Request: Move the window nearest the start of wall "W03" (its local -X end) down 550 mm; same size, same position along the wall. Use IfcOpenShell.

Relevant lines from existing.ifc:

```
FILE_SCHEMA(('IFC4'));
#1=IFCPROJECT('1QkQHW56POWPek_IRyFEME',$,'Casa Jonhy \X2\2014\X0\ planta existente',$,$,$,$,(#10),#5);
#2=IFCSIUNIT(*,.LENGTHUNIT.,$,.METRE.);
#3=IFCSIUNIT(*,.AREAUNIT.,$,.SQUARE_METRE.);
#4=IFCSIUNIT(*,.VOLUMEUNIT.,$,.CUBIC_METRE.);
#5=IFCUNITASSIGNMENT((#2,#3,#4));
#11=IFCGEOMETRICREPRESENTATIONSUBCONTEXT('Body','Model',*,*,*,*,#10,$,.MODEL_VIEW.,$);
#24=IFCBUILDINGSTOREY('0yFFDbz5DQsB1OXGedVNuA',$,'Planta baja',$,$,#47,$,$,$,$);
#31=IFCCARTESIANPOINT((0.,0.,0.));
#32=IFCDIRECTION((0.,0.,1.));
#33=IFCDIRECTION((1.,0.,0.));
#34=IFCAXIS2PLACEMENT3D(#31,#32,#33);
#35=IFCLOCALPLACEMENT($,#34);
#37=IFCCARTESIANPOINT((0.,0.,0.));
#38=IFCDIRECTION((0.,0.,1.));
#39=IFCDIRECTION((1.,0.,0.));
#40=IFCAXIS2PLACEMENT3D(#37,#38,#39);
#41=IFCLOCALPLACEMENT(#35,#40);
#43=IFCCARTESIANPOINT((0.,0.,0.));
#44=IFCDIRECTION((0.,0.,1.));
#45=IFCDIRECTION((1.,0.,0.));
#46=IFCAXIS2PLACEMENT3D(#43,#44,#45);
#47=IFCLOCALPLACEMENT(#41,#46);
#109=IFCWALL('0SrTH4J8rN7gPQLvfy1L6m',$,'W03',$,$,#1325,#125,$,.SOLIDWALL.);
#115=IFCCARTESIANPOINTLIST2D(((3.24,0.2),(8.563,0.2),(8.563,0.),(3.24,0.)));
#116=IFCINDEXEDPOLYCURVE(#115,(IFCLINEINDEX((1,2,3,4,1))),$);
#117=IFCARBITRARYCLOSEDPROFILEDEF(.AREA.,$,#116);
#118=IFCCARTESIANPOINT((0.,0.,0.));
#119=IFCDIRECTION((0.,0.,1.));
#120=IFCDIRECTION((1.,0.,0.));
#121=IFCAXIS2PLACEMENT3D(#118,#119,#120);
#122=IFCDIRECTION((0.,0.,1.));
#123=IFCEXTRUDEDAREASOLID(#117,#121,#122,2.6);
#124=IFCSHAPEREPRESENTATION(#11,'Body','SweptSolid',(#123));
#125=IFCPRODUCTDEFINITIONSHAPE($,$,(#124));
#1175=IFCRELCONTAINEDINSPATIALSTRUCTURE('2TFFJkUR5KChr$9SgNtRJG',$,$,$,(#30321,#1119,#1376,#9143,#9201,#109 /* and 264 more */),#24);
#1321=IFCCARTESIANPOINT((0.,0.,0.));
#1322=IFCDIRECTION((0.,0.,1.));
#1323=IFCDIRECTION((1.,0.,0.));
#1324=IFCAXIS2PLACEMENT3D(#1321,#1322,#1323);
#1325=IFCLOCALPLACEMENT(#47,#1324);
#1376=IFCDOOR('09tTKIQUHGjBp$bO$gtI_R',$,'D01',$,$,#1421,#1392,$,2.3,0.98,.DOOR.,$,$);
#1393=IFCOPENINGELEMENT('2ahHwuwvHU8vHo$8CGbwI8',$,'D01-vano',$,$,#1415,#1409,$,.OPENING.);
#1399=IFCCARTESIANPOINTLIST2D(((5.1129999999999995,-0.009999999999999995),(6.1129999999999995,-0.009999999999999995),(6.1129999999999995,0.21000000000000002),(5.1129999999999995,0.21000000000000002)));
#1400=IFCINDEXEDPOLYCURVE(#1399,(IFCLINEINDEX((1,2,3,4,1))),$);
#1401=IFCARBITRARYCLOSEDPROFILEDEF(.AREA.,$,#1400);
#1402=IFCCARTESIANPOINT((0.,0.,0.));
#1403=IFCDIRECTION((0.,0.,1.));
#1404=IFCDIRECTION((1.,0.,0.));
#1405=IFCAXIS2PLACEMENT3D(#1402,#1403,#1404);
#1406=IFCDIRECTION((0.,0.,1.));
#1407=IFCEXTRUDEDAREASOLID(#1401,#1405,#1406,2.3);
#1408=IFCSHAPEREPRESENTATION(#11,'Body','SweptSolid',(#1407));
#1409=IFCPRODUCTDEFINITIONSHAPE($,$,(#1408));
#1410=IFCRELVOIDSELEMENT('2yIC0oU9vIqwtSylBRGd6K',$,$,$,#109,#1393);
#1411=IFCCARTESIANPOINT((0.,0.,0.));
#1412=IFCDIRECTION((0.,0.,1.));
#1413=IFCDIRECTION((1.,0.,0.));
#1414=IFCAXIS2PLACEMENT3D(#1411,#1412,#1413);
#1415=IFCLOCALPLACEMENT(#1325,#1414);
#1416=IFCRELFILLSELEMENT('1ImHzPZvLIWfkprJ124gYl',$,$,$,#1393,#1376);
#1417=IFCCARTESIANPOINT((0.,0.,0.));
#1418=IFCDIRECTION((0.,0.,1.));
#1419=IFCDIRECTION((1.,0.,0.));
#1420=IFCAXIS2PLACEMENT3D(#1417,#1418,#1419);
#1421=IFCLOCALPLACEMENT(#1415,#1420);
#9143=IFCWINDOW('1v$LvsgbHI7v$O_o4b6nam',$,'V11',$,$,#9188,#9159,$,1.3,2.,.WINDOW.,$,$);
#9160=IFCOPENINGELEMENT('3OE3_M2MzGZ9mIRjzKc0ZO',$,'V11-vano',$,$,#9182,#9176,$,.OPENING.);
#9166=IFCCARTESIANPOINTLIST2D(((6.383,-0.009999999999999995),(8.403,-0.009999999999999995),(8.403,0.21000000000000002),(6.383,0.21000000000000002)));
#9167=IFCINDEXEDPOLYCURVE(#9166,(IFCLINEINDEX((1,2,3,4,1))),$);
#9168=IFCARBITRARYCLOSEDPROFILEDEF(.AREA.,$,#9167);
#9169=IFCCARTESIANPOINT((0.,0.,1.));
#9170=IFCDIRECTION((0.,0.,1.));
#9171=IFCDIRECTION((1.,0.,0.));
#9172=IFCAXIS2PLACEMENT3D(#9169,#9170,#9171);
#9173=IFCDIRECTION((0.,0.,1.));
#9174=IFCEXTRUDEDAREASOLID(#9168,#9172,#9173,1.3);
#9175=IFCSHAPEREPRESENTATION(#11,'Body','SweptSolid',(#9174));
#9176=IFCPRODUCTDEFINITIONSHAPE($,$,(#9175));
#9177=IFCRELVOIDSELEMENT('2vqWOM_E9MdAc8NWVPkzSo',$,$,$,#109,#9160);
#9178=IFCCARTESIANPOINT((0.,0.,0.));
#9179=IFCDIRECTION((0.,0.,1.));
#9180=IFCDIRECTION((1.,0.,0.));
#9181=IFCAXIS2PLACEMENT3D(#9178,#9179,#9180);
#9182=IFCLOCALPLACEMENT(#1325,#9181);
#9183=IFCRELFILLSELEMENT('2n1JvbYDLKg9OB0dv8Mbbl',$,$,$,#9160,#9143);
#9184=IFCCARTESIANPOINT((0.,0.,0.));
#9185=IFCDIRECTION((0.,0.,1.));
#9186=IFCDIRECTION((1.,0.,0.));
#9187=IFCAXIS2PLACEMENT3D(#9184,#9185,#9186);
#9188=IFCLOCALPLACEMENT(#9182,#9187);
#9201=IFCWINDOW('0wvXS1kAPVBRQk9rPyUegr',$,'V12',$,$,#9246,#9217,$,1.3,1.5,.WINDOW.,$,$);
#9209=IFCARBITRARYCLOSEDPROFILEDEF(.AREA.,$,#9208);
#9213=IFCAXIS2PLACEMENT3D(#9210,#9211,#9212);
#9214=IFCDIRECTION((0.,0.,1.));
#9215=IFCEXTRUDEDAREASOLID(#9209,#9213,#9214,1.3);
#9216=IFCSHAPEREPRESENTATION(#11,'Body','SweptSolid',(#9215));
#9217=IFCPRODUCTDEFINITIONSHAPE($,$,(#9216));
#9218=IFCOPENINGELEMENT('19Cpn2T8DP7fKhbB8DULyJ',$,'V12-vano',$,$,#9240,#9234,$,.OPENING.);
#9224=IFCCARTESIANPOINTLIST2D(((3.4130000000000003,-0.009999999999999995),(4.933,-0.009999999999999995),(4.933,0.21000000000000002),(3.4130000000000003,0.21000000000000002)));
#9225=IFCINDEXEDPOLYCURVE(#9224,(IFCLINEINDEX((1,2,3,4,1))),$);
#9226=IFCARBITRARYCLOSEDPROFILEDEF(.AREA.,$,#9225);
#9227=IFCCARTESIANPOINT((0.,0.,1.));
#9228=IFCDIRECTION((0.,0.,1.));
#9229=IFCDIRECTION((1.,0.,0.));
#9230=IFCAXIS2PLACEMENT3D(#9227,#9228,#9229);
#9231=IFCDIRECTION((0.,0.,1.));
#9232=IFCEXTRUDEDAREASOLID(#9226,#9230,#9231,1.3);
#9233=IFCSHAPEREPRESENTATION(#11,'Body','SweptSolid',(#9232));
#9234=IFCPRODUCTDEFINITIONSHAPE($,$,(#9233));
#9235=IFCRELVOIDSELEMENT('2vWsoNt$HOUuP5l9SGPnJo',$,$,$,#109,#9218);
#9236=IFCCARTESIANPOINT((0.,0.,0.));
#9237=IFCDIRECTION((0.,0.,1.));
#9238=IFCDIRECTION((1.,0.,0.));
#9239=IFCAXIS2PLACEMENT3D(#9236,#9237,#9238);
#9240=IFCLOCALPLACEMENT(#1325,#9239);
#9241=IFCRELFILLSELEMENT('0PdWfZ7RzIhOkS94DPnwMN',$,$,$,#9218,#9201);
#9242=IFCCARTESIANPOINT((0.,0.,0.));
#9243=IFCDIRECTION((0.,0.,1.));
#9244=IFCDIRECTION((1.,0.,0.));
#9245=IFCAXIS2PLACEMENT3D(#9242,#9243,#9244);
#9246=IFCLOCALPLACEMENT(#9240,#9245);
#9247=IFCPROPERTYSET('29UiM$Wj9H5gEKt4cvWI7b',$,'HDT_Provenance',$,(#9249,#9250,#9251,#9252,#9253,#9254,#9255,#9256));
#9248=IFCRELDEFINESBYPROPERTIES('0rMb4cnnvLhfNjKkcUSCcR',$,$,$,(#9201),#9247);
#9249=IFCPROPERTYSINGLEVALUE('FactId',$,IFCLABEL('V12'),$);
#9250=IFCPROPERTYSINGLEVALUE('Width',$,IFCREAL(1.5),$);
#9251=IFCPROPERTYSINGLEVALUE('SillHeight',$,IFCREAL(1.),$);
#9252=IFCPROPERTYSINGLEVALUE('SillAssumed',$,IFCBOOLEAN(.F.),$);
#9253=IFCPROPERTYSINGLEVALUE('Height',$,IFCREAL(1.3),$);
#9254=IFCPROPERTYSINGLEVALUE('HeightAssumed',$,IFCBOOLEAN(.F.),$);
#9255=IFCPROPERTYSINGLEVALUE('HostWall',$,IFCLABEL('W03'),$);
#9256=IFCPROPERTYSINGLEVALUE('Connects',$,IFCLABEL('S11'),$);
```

```python
import numpy as np
import ifcopenshell
import ifcopenshell.api.geometry
import ifcopenshell.api.pset
import ifcopenshell.util.element
import ifcopenshell.util.placement
import ifcopenshell.util.unit

model = ifcopenshell.open("existing.ifc")
unit_scale = ifcopenshell.util.unit.calculate_unit_scale(model)

window = model.by_guid("0wvXS1kAPVBRQk9rPyUegr")
opening = window.FillsVoids[0].RelatingOpeningElement
dz = -0.55 / unit_scale

shift = np.array([0.0, 0.0, dz])
# The window is placed relative to its opening, so it follows when the opening moves.
matrix = ifcopenshell.util.placement.get_local_placement(opening.ObjectPlacement)
matrix[:3, 3] += shift
ifcopenshell.api.geometry.edit_object_placement(
    model, product=opening, matrix=matrix, is_si=False, should_transform_children=True
)

# Keep the stored heights in step.
pset = model.by_id(ifcopenshell.util.element.get_pset(window, "HDT_Provenance", should_inherit=False)["id"])
ifcopenshell.api.pset.edit_pset(model, pset=pset, properties={
    "SillHeight": model.create_entity("IfcReal", ifcopenshell.util.element.get_pset(window, "HDT_Provenance", "SillHeight") + dz),
})

print(f"moved by {dz * unit_scale:+.3f} m")

model.write("existing_updated.ifc")
```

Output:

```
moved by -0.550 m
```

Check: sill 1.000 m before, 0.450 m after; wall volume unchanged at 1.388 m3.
